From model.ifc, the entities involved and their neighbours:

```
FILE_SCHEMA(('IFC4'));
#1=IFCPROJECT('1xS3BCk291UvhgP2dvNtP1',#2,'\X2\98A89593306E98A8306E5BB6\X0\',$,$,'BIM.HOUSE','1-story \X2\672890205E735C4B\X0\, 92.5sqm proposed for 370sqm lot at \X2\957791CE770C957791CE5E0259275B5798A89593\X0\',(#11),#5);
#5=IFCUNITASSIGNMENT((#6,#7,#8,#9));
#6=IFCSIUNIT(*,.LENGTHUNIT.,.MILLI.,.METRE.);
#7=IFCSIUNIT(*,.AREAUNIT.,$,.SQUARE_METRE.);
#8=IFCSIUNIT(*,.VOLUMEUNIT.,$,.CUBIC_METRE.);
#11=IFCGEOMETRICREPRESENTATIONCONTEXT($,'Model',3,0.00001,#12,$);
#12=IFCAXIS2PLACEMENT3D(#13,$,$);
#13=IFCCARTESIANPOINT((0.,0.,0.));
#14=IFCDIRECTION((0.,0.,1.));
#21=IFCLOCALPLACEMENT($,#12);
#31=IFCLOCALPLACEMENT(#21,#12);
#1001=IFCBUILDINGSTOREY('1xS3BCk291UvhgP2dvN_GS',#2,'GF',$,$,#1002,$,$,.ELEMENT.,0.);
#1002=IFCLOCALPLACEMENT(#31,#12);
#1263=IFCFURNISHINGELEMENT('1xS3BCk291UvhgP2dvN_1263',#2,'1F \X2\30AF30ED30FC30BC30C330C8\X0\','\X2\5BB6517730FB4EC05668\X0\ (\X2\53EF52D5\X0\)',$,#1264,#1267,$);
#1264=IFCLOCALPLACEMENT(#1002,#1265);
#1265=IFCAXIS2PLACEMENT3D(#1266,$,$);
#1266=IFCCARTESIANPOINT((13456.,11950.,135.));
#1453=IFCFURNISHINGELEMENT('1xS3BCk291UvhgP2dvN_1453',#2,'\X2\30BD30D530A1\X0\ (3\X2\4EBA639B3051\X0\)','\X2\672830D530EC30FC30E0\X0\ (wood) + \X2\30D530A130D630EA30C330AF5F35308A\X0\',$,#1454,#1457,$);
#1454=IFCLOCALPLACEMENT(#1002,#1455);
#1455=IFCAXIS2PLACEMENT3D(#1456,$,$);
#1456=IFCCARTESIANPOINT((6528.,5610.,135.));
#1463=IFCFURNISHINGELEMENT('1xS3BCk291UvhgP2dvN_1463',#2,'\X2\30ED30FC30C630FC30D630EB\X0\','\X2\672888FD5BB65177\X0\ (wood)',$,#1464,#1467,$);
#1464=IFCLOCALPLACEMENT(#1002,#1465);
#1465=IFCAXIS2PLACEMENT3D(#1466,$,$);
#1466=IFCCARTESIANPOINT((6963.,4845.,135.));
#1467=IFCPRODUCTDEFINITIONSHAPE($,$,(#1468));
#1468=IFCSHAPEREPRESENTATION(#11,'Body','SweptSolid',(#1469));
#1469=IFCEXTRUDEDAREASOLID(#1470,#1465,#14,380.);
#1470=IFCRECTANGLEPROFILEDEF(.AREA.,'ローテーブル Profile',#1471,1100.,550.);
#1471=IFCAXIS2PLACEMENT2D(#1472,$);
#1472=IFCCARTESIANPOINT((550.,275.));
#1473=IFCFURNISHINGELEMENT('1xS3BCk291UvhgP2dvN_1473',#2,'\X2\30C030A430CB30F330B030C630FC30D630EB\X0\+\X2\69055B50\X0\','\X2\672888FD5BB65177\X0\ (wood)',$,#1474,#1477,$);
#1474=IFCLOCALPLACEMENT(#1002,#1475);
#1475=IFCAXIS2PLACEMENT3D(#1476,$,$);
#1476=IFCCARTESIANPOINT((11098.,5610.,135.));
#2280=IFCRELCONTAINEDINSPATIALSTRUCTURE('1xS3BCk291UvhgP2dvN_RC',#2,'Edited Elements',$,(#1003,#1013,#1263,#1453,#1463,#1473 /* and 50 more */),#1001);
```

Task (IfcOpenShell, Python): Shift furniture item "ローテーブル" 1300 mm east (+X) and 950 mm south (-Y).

```python
import ifcopenshell
import ifcopenshell.api.geometry
import ifcopenshell.util.placement
import ifcopenshell.util.unit

model = ifcopenshell.open("model.ifc")
unit_scale = ifcopenshell.util.unit.calculate_unit_scale(model)

item = model.by_guid("1xS3BCk291UvhgP2dvN_1463")
matrix = ifcopenshell.util.placement.get_local_placement(item.ObjectPlacement)
matrix[0, 3] += 1.3 / unit_scale
matrix[1, 3] -= 0.95 / unit_scale
ifcopenshell.api.geometry.edit_object_placement(model, product=item, matrix=matrix, is_si=False)

print(ifcopenshell.util.placement.get_local_placement(item.ObjectPlacement).round(3) + 0.0)

model.write("model_edited.ifc")
```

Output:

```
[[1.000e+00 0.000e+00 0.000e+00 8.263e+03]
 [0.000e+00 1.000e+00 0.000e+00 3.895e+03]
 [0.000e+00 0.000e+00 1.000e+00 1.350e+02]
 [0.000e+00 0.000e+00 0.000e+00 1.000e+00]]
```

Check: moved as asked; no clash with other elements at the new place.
